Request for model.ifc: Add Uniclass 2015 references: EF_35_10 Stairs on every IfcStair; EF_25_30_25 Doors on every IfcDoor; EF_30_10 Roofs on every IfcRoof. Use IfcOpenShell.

First a look at what the model holds.

```python
import ifcopenshell

model = ifcopenshell.open("model.ifc")
print(model.schema)
print("classifications:", [c.Name for c in model.by_type("IfcClassification")])
for ifc_class in ("IfcDoor", "IfcRoof", "IfcStair", "IfcWall", "IfcWindow"):
    print(ifc_class, len(model.by_type(ifc_class)))
```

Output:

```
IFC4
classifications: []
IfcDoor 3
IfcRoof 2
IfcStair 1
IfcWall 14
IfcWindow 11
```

```python
import ifcopenshell
import ifcopenshell.api.classification

model = ifcopenshell.open("model.ifc")

system = ifcopenshell.api.classification.add_classification(model, classification="Uniclass 2015")

codes = {
    "IfcStair": ("EF_35_10", "Stairs"),
    "IfcDoor": ("EF_25_30_25", "Doors"),
    "IfcRoof": ("EF_30_10", "Roofs"),
}
for ifc_class, (code, name) in codes.items():
    products = model.by_type(ifc_class)
    ifcopenshell.api.classification.add_reference(
        model, products=products, classification=system, identification=code, name=name
    )
    print(code, len(products))

model.write("model_rev.ifc")
```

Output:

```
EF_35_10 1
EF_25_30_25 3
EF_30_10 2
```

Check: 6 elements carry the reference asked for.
